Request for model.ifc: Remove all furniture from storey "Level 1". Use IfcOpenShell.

First a look at what the model holds.

```python
import ifcopenshell
import ifcopenshell.util.element

model = ifcopenshell.open("model.ifc")
print(model.schema)
storey = next(s for s in model.by_type("IfcBuildingStorey") if s.Name == "Level 1")
furniture = [e for e in ifcopenshell.util.element.get_decomposition(storey) if e.is_a("IfcFurnishingElement")]
seen = {}
for e in furniture:
    element_type = ifcopenshell.util.element.get_type(e)
    name = element_type.Name if element_type not in (None, e) else None
    seen[name] = seen.get(name, 0) + 1
for name, count in sorted(seen.items(), key=str):
    print(count, "x", name)
```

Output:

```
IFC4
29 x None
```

```python
import ifcopenshell
import ifcopenshell.api.root
import ifcopenshell.util.element

model = ifcopenshell.open("model.ifc")

storey = next(s for s in model.by_type("IfcBuildingStorey") if s.Name == "Level 1")
furniture = [e for e in ifcopenshell.util.element.get_decomposition(storey) if e.is_a("IfcFurnishingElement")]

for e in furniture:
    ifcopenshell.api.root.remove_product(model, product=e)
print(len(furniture), "removed")

model.write("model_edited.ifc")
```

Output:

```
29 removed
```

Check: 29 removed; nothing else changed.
